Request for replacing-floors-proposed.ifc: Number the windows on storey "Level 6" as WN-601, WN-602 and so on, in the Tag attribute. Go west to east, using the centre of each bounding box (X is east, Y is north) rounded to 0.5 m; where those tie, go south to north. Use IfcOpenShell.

First a look at what the model holds.

```python
import ifcopenshell
import ifcopenshell.util.element
import ifcopenshell.util.placement

model = ifcopenshell.open("replacing-floors-proposed.ifc")
print(model.schema)
storey = next(s for s in model.by_type("IfcBuildingStorey") if s.Name == "Level 6")
windows = [e for e in ifcopenshell.util.element.get_decomposition(storey) if e.is_a("IfcWindow")]
for e in sorted(windows, key=lambda e: e.id()):
    origin = ifcopenshell.util.placement.get_local_placement(e.ObjectPlacement)[:3, 3]
    print(e.id(), e.Tag, e.Name, origin.round(2) + 0.0, sep=" | ")
```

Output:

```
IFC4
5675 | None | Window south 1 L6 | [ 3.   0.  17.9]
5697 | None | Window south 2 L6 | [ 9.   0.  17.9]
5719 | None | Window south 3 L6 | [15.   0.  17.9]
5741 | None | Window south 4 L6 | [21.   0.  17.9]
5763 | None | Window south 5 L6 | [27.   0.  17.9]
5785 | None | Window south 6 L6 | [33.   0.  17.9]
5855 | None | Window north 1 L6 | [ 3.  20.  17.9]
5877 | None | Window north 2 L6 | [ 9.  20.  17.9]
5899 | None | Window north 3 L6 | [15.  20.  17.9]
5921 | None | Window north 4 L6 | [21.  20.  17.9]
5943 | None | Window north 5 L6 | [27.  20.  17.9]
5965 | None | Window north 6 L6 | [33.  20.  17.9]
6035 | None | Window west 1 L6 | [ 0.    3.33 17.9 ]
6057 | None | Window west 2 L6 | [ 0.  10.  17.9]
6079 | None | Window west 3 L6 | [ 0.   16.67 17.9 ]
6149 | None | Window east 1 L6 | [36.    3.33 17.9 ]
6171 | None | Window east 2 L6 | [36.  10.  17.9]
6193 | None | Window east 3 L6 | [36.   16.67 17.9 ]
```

```python
import ifcopenshell
import ifcopenshell.geom
import ifcopenshell.util.element
import ifcopenshell.util.shape

model = ifcopenshell.open("replacing-floors-proposed.ifc")
settings = ifcopenshell.geom.settings()
settings.set("use-world-coords", True)


def centre(element):
    shape = ifcopenshell.geom.create_shape(settings, element)
    return ifcopenshell.util.shape.get_bbox_centroid(shape.geometry)


storey = next(s for s in model.by_type("IfcBuildingStorey") if s.Name == "Level 6")
windows = [e for e in ifcopenshell.util.element.get_decomposition(storey) if e.is_a("IfcWindow")]

# Insertion points can sit at a corner or the storey origin, so sort by the geometry (in metres).
centres = {e: centre(e) for e in windows}
windows.sort(key=lambda e: (round(centres[e][0] / 0.5), centres[e][1]))

for i, e in enumerate(windows, start=1):
    number = f"WN-6{i:02d}"
    e.Tag = number
    print(e.id(), number)

model.write("replacing-floors-proposed_edited.ifc")
```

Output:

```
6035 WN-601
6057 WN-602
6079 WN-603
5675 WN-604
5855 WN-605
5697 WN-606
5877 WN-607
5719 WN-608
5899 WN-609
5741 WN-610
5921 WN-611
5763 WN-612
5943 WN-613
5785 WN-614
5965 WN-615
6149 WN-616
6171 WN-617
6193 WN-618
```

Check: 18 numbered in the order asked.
